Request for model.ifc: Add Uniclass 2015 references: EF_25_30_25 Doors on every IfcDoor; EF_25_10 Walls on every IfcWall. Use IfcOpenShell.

First a look at what the model holds.

```python
import ifcopenshell

model = ifcopenshell.open("model.ifc")
print(model.schema)
print("classifications:", [c.Name for c in model.by_type("IfcClassification")])
for ifc_class in ("IfcDoor", "IfcRoof", "IfcStair", "IfcWall", "IfcWindow"):
    print(ifc_class, len(model.by_type(ifc_class)))
```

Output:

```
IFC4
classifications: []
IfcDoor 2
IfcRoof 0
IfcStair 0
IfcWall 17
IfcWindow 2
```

```python
import ifcopenshell
import ifcopenshell.api.classification

model = ifcopenshell.open("model.ifc")

system = ifcopenshell.api.classification.add_classification(model, classification="Uniclass 2015")

codes = {
    "IfcDoor": ("EF_25_30_25", "Doors"),
    "IfcWall": ("EF_25_10", "Walls"),
}
for ifc_class, (code, name) in codes.items():
    products = model.by_type(ifc_class)
    ifcopenshell.api.classification.add_reference(
        model, products=products, classification=system, identification=code, name=name
    )
    print(code, len(products))

model.write("model_v2.ifc")
```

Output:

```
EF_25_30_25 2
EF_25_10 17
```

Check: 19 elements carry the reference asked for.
